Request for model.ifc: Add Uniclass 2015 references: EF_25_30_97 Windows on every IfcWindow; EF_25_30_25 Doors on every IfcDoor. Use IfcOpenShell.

First a look at what the model holds.

```python
import ifcopenshell

model = ifcopenshell.open("model.ifc")
print(model.schema)
print("classifications:", [c.Name for c in model.by_type("IfcClassification")])
for ifc_class in ("IfcDoor", "IfcRoof", "IfcStair", "IfcWall", "IfcWindow"):
    print(ifc_class, len(model.by_type(ifc_class)))
```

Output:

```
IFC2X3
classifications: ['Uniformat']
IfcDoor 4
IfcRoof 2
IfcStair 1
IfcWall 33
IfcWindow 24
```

```python
import ifcopenshell
import ifcopenshell.api.classification

model = ifcopenshell.open("model.ifc")

# IFC2X3 requires Source and Edition and has no link from the project to the system.
system = model.create_entity("IfcClassification", Source="NBS", Edition="2015", Name="Uniclass 2015")

codes = {
    "IfcWindow": ("EF_25_30_97", "Windows"),
    "IfcDoor": ("EF_25_30_25", "Doors"),
}
for ifc_class, (code, name) in codes.items():
    products = model.by_type(ifc_class)
    ifcopenshell.api.classification.add_reference(
        model, products=products, classification=system, identification=code, name=name
    )
    print(code, len(products))

model.write("model_updated.ifc")
```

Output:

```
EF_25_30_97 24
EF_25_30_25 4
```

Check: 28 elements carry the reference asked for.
